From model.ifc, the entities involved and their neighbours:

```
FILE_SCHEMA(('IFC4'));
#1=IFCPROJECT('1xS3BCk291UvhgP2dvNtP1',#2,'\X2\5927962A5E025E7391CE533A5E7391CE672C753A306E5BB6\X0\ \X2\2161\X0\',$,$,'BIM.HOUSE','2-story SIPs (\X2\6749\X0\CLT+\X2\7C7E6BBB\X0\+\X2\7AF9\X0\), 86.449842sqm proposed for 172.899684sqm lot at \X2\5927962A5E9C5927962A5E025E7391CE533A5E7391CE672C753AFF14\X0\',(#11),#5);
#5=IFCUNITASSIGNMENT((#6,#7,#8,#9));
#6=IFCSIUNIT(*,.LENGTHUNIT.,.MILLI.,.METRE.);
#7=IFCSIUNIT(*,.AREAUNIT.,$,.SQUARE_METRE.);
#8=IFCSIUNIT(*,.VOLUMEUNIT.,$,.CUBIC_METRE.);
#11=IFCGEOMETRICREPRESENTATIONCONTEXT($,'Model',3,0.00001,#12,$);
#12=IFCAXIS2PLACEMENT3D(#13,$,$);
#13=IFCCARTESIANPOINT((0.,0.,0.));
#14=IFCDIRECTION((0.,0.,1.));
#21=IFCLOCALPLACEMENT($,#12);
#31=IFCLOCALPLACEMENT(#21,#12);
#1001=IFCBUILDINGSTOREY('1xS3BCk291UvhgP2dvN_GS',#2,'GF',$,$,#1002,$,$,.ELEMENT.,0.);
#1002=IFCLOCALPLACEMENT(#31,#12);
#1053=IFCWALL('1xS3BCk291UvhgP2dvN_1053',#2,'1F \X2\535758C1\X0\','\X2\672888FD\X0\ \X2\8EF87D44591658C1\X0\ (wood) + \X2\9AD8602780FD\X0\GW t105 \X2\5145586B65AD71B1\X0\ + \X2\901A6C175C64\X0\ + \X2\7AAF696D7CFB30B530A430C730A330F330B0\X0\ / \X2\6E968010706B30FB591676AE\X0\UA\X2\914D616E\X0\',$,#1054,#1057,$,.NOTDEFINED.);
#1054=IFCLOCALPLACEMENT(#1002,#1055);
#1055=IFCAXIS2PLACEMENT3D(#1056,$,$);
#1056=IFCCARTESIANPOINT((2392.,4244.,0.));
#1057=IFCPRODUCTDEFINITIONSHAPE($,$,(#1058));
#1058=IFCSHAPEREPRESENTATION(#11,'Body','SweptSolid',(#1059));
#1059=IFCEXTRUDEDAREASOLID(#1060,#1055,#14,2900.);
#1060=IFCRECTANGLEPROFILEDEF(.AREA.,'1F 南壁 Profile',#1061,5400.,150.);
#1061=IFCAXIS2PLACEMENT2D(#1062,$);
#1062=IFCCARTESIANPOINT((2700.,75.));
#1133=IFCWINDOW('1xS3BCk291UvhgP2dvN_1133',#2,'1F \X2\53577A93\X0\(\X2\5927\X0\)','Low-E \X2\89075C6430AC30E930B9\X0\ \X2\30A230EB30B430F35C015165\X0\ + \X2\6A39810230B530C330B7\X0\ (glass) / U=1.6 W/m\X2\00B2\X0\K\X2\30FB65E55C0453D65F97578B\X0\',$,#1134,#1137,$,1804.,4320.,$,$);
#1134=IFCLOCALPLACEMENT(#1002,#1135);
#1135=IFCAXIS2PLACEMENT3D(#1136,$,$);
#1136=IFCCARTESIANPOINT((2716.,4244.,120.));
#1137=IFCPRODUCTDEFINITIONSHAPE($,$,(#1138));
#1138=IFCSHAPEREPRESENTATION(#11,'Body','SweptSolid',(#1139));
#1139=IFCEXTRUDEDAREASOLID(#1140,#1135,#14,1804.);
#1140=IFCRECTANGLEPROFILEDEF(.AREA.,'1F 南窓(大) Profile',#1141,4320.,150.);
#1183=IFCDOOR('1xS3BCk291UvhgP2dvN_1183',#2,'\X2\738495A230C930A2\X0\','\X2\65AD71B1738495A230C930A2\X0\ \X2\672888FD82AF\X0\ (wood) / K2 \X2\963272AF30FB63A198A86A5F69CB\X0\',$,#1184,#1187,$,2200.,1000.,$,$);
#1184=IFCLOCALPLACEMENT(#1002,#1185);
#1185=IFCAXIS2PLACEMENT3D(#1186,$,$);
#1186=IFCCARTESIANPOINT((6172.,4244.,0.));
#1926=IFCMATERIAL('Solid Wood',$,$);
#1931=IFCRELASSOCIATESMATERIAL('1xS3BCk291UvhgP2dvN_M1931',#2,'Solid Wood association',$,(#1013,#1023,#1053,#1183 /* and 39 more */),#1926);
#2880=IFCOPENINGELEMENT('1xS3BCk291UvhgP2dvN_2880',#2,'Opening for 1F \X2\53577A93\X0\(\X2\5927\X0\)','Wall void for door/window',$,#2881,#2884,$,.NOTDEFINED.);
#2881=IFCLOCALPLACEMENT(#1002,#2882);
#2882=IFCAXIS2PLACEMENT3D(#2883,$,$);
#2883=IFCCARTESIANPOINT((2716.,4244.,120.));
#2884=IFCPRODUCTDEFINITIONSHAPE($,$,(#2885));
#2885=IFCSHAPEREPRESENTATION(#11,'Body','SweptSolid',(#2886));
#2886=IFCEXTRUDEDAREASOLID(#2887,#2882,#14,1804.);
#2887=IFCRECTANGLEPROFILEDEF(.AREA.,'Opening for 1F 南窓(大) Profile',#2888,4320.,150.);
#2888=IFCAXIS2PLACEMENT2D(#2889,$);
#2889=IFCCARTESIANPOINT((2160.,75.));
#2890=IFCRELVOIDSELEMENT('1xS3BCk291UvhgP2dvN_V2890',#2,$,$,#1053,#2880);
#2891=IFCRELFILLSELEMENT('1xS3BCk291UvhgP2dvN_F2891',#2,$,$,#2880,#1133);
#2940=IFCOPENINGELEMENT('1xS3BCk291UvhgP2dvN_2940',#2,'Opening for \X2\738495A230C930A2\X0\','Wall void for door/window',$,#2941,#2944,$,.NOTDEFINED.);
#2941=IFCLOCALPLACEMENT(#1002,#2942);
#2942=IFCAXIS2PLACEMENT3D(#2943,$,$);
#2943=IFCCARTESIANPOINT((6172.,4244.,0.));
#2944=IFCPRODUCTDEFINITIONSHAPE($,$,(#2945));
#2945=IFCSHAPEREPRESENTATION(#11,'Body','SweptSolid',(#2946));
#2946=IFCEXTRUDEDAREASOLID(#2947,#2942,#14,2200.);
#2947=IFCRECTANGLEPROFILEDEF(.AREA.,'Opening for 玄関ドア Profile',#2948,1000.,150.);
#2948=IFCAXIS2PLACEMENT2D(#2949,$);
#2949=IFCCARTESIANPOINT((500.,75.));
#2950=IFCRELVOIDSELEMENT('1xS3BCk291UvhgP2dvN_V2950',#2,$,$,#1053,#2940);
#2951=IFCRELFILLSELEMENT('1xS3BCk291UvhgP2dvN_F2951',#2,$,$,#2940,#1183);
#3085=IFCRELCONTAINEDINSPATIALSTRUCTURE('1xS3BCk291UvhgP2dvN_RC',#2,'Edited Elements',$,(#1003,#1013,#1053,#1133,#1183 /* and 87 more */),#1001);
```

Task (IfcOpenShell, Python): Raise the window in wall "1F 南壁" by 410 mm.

```python
import numpy as np
import ifcopenshell
import ifcopenshell.api.geometry
import ifcopenshell.util.placement
import ifcopenshell.util.unit

model = ifcopenshell.open("model.ifc")
unit_scale = ifcopenshell.util.unit.calculate_unit_scale(model)

window = model.by_id(1133)
opening = window.FillsVoids[0].RelatingOpeningElement
dz = 0.41 / unit_scale

shift = np.array([0.0, 0.0, dz])
# The window is not placed relative to its opening, so move both.
for product in (opening, window):
    matrix = ifcopenshell.util.placement.get_local_placement(product.ObjectPlacement)
    matrix[:3, 3] += shift
    ifcopenshell.api.geometry.edit_object_placement(model, product=product, matrix=matrix, is_si=False)

print(f"moved by {dz * unit_scale:+.3f} m")

model.write("model_v2.ifc")
```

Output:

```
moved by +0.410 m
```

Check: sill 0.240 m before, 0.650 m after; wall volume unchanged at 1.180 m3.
